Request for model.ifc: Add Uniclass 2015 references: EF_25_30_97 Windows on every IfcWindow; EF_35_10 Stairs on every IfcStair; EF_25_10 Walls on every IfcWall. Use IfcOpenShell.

First a look at what the model holds.

```python
import ifcopenshell

model = ifcopenshell.open("model.ifc")
print(model.schema)
print("classifications:", [c.Name for c in model.by_type("IfcClassification")])
for ifc_class in ("IfcDoor", "IfcRoof", "IfcStair", "IfcWall", "IfcWindow"):
    print(ifc_class, len(model.by_type(ifc_class)))
```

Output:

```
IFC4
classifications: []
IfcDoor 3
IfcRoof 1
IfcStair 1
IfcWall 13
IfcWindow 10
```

```python
import ifcopenshell
import ifcopenshell.api.classification

model = ifcopenshell.open("model.ifc")

system = ifcopenshell.api.classification.add_classification(model, classification="Uniclass 2015")

codes = {
    "IfcWindow": ("EF_25_30_97", "Windows"),
    "IfcStair": ("EF_35_10", "Stairs"),
    "IfcWall": ("EF_25_10", "Walls"),
}
for ifc_class, (code, name) in codes.items():
    products = model.by_type(ifc_class)
    ifcopenshell.api.classification.add_reference(
        model, products=products, classification=system, identification=code, name=name
    )
    print(code, len(products))

model.write("model_rev.ifc")
```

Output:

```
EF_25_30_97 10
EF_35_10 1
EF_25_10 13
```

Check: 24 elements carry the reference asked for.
